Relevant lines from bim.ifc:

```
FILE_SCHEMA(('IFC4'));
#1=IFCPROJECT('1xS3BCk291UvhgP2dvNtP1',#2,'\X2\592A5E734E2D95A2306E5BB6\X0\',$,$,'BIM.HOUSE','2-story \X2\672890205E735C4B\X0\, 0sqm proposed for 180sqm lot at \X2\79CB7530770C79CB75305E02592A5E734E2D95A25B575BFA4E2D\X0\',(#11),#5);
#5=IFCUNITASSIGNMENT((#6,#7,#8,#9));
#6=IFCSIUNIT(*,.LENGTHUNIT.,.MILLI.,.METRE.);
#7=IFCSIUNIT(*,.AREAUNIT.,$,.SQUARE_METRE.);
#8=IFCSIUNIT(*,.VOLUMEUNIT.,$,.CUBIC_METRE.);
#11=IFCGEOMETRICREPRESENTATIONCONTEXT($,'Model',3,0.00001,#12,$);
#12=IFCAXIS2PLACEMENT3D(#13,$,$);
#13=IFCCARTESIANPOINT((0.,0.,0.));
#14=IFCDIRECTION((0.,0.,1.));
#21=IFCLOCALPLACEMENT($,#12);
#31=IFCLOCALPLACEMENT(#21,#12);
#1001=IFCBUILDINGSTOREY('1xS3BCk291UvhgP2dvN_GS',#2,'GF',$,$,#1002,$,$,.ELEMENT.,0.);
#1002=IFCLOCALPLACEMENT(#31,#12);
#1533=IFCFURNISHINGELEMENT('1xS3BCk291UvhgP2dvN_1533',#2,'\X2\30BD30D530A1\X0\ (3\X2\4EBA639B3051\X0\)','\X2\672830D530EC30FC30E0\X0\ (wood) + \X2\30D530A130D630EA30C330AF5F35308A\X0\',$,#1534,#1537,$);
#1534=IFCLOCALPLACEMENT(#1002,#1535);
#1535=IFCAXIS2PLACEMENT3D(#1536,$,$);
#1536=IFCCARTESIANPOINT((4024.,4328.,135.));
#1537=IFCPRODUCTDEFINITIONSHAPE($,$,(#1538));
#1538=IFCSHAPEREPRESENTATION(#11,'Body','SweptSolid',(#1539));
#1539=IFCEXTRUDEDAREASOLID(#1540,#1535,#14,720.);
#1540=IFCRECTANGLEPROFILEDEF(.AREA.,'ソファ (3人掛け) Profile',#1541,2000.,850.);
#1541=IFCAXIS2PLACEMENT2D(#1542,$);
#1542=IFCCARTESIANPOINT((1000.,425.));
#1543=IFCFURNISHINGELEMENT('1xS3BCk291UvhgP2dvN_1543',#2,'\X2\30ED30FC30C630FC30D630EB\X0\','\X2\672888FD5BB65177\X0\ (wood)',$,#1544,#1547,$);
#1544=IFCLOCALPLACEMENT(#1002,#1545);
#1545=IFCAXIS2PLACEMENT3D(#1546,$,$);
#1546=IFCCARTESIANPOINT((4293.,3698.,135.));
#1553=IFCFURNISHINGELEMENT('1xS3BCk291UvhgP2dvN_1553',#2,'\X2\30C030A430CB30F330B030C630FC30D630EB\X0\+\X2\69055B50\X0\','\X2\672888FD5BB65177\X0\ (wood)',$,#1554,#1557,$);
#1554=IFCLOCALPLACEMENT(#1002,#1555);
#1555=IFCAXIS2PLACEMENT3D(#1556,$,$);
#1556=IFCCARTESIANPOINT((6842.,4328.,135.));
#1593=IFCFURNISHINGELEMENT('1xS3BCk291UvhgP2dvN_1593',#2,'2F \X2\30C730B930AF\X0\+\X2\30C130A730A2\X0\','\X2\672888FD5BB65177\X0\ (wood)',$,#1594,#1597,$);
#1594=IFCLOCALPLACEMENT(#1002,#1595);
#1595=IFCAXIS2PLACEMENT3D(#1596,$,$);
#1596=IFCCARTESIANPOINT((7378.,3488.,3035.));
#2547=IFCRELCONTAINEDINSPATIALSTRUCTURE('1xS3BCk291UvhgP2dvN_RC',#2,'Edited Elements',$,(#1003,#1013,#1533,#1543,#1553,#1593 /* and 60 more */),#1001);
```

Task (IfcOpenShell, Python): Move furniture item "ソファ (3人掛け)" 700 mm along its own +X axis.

```python
import ifcopenshell
import ifcopenshell.api.geometry
import ifcopenshell.util.placement
import ifcopenshell.util.unit

model = ifcopenshell.open("bim.ifc")
unit_scale = ifcopenshell.util.unit.calculate_unit_scale(model)

item = model.by_id(1533)
matrix = ifcopenshell.util.placement.get_local_placement(item.ObjectPlacement)
matrix[:3, 3] += matrix[:3, 0] * 0.7 / unit_scale
ifcopenshell.api.geometry.edit_object_placement(model, product=item, matrix=matrix, is_si=False)

print(ifcopenshell.util.placement.get_local_placement(item.ObjectPlacement).round(3) + 0.0)

model.write("bim_rev.ifc")
```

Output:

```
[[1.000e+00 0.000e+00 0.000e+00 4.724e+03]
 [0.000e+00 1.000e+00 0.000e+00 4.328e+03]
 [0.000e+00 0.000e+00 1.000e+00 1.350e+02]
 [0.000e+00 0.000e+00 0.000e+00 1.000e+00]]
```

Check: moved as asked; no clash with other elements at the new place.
